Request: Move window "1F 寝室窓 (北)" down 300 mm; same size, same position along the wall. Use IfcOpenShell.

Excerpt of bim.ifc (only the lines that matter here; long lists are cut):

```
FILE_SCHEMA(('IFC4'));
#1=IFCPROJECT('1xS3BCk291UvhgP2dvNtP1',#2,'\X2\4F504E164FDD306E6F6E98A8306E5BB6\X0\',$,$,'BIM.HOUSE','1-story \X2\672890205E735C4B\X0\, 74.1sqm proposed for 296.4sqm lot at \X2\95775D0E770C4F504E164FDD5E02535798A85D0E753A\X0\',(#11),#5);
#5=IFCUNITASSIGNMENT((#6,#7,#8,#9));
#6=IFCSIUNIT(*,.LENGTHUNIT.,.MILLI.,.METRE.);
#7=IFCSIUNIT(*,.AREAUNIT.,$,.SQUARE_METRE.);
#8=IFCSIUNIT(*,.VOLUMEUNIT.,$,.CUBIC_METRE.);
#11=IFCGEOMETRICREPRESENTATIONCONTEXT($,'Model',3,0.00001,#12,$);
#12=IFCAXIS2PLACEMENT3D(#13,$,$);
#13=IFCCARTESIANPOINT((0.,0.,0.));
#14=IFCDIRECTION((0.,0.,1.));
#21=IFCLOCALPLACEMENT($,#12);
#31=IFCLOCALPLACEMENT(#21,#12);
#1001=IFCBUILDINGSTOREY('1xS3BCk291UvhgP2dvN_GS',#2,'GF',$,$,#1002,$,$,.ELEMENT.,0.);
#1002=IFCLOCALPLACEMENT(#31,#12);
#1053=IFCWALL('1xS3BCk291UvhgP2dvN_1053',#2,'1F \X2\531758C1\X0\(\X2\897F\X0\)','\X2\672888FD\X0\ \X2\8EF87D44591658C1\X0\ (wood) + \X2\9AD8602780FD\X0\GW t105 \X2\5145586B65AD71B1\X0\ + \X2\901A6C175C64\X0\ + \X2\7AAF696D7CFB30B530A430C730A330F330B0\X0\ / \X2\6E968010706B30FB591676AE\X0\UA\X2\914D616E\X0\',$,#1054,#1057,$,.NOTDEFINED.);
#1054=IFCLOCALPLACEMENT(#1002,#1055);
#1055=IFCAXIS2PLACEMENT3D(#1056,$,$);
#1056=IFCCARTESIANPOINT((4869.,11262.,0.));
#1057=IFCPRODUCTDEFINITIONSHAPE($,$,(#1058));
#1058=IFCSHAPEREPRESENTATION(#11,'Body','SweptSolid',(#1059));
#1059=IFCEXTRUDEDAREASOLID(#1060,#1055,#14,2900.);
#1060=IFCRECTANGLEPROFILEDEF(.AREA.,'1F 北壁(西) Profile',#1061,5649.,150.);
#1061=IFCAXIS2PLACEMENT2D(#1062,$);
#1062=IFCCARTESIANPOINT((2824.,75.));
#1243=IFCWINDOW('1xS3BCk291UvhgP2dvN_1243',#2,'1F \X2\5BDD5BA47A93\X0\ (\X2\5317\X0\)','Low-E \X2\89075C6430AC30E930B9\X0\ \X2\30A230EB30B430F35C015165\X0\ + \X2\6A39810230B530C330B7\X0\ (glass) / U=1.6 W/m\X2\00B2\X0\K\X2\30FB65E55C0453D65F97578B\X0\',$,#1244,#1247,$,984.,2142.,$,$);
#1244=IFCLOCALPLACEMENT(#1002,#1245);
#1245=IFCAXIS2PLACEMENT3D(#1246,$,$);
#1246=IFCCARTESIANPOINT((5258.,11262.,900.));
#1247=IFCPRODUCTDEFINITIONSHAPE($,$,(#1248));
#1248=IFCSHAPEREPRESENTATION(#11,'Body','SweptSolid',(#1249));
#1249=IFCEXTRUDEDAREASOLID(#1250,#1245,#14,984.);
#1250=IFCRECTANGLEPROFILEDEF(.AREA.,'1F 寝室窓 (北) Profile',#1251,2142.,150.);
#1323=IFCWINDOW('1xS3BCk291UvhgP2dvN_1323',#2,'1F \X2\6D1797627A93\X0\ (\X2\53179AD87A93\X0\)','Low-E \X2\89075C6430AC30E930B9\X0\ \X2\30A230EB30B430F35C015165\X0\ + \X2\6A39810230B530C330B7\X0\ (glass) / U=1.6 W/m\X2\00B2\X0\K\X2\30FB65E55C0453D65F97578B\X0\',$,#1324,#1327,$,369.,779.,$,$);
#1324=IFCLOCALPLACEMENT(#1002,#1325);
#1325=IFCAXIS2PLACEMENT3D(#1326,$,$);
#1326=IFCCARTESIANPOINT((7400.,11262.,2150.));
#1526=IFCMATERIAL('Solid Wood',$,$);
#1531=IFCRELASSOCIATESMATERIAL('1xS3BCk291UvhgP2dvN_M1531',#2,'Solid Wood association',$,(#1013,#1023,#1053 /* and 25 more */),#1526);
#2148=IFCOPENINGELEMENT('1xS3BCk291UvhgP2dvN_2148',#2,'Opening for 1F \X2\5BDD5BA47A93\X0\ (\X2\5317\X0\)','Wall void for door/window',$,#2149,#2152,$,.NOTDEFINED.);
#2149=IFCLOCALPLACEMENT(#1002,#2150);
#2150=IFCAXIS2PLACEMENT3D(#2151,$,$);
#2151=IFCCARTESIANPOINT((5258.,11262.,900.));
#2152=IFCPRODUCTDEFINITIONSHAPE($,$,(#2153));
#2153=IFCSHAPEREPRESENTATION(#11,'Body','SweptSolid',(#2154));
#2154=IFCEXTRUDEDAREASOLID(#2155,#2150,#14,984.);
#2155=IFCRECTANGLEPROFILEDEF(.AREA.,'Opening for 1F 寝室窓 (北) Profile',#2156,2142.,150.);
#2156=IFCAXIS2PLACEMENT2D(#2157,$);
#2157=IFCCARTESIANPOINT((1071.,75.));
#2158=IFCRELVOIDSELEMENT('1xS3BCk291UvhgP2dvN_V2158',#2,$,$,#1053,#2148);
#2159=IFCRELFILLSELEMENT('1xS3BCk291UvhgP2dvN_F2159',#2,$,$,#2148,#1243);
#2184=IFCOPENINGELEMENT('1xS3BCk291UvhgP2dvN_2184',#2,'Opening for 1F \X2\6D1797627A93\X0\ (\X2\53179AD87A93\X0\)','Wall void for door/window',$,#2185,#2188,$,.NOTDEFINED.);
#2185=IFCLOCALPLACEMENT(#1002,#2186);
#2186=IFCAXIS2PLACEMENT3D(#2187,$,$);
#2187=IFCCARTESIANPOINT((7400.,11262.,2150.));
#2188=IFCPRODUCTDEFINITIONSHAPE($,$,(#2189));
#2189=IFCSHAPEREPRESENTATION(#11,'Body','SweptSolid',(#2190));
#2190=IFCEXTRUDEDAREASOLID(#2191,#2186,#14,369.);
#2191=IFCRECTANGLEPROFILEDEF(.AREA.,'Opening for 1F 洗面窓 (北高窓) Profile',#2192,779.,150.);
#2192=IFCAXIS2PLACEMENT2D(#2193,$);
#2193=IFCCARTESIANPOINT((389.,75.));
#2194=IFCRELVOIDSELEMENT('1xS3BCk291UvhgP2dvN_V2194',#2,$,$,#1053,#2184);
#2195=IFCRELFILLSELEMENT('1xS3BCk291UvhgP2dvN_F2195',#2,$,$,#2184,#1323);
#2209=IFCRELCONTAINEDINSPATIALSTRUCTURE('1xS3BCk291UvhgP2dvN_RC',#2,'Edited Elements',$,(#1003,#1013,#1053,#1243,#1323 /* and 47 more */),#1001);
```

```python
import numpy as np
import ifcopenshell
import ifcopenshell.api.geometry
import ifcopenshell.util.placement
import ifcopenshell.util.unit

model = ifcopenshell.open("bim.ifc")
unit_scale = ifcopenshell.util.unit.calculate_unit_scale(model)

window = model.by_guid("1xS3BCk291UvhgP2dvN_1243")
opening = window.FillsVoids[0].RelatingOpeningElement
dz = -0.3 / unit_scale

shift = np.array([0.0, 0.0, dz])
# The window is not placed relative to its opening, so move both.
for product in (opening, window):
    matrix = ifcopenshell.util.placement.get_local_placement(product.ObjectPlacement)
    matrix[:3, 3] += shift
    ifcopenshell.api.geometry.edit_object_placement(model, product=product, matrix=matrix, is_si=False)

print(f"moved by {dz * unit_scale:+.3f} m")

model.write("bim-out.ifc")
```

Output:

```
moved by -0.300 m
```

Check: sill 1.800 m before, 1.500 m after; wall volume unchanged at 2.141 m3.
